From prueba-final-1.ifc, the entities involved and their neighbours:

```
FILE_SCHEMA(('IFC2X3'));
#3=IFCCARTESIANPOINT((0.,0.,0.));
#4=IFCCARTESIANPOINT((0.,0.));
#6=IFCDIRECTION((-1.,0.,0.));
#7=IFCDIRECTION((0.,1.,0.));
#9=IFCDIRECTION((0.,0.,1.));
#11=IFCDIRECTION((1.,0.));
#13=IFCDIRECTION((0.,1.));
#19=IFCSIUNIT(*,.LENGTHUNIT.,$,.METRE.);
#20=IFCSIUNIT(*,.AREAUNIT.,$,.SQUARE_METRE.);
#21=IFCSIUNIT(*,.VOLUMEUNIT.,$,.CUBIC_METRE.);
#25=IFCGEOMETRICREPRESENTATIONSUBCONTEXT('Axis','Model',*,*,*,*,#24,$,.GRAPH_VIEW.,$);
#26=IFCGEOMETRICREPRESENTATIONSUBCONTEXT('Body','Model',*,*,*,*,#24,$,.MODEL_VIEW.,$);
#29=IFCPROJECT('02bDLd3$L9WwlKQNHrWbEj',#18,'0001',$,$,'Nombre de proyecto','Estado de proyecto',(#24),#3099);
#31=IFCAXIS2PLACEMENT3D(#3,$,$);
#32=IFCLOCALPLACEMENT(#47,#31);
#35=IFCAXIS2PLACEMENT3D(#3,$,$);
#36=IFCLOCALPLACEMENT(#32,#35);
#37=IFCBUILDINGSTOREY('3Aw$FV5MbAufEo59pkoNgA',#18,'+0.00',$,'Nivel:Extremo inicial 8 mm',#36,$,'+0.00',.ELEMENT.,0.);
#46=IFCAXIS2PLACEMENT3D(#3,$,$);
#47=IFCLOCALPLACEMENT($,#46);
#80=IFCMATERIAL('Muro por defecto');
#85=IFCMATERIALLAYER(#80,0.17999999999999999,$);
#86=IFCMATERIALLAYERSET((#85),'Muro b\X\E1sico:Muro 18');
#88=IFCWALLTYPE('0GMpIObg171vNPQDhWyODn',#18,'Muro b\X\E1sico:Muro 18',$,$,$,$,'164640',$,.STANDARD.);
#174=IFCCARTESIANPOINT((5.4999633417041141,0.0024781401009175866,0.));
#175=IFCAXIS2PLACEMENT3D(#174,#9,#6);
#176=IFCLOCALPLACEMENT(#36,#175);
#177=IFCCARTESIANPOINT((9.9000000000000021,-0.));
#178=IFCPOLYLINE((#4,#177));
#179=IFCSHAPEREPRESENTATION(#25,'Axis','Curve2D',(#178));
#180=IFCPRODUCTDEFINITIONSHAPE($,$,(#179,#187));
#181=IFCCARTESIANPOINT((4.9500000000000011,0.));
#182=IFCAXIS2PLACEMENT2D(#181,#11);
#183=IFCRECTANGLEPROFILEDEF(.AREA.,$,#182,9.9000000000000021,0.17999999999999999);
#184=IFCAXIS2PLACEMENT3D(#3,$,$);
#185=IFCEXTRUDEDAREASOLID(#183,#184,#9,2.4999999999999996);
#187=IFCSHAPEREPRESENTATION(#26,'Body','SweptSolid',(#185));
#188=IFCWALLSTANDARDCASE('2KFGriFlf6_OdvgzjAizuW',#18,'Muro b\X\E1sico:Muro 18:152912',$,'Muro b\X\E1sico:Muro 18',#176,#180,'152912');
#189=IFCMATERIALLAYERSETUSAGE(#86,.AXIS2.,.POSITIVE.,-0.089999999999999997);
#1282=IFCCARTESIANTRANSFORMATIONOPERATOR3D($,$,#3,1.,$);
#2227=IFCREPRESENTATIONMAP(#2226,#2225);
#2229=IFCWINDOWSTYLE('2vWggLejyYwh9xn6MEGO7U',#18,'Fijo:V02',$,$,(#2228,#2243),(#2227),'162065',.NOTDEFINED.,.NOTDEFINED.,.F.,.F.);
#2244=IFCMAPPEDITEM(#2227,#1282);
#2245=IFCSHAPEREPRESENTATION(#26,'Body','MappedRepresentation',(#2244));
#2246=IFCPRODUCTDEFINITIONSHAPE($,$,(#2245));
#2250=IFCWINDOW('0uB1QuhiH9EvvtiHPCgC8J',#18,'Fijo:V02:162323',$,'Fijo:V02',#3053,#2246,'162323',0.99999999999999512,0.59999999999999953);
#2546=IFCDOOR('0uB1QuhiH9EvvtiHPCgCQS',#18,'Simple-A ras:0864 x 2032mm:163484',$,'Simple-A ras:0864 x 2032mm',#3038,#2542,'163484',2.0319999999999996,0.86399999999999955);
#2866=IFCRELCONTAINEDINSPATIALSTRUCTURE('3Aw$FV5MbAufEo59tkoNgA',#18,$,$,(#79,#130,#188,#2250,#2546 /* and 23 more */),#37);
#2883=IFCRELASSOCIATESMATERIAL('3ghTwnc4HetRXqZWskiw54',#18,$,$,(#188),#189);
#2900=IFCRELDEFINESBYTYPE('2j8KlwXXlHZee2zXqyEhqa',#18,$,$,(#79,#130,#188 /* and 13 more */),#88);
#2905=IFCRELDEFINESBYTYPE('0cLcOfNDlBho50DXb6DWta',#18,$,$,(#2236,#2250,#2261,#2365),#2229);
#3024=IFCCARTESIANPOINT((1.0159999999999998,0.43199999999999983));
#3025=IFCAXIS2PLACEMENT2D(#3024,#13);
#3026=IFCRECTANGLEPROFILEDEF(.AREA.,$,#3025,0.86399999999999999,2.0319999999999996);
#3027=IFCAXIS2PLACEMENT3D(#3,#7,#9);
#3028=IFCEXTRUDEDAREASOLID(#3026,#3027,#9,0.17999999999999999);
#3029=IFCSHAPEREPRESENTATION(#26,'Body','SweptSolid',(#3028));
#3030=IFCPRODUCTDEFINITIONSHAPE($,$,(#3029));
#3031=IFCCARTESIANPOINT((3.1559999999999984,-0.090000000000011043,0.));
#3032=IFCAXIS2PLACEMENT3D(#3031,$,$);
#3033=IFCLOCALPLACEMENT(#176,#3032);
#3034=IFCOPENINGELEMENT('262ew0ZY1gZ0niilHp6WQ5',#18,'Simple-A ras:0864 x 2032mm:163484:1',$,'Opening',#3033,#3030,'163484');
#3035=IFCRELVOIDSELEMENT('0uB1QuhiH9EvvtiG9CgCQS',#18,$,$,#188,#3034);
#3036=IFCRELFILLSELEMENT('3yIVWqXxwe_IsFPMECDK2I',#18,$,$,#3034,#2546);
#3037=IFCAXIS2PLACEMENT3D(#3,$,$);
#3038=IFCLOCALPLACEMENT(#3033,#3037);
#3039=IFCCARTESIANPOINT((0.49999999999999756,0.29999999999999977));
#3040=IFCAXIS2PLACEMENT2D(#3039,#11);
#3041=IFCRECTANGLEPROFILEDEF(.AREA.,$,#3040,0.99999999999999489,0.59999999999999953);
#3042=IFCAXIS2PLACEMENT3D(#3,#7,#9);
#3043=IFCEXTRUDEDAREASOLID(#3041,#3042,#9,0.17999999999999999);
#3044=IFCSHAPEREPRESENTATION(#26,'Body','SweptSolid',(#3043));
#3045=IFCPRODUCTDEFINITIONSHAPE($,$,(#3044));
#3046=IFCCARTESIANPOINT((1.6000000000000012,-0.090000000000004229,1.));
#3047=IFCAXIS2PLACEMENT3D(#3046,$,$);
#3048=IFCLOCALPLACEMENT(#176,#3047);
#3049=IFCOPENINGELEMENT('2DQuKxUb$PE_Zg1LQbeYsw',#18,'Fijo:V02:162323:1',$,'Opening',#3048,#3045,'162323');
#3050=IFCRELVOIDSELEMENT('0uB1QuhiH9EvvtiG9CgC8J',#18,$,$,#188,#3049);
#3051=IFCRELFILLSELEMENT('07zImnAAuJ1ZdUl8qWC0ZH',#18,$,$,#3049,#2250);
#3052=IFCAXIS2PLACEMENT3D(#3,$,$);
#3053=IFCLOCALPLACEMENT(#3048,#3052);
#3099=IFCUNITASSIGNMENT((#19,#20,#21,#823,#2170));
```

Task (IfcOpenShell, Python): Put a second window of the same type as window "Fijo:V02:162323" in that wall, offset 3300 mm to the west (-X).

```python
import ifcopenshell
import ifcopenshell.api.feature
import ifcopenshell.api.geometry
import ifcopenshell.api.root
import ifcopenshell.geom
import ifcopenshell.util.element
import ifcopenshell.util.placement
import ifcopenshell.util.shape

model = ifcopenshell.open("prueba-final-1.ifc")
settings = ifcopenshell.geom.settings()


def volume(element):
    """Net volume in cubic metres, openings subtracted."""
    shape = ifcopenshell.geom.create_shape(settings, element)
    return ifcopenshell.util.shape.get_volume(shape.geometry)


def reuse_history(source, copy):
    """copy_class also copies each property set's owner history, people and application; keep the originals."""
    for rel in copy.IsDefinedBy:
        if rel.is_a("IfcRelDefinesByProperties") and (history := rel.RelatingPropertyDefinition.OwnerHistory):
            rel.RelatingPropertyDefinition.OwnerHistory = source.OwnerHistory
            ifcopenshell.util.element.remove_deep2(model, history)


window = model.by_id(2250)
opening = window.FillsVoids[0].RelatingOpeningElement
wall = opening.VoidsElements[0].RelatingBuildingElement
before = volume(wall)
shift = ifcopenshell.util.placement.get_local_placement(wall.ObjectPlacement)[:3, 0] * 3.3

# copy_class copies the void relationship, type, container and properties, but no geometry.
new_opening = ifcopenshell.api.root.copy_class(model, product=opening)
new_opening.Representation = ifcopenshell.util.element.copy_deep(
    model, opening.Representation, exclude=["IfcGeometricRepresentationContext", "IfcRepresentationMap"]
)
new_opening.Name = "Fijo:V02"
new_opening.Tag = None
new_window = ifcopenshell.api.root.copy_class(model, product=window)
new_window.Representation = ifcopenshell.util.element.copy_deep(
    model, window.Representation, exclude=["IfcGeometricRepresentationContext", "IfcRepresentationMap"]
)
new_window.Name = "Fijo:V02"
new_window.Tag = None
reuse_history(window, new_window)
fills = ifcopenshell.api.feature.add_filling(model, opening=new_opening, element=new_window)
fills.OwnerHistory = new_window.OwnerHistory  # required in IFC2X3

for old, new in ((opening, new_opening), (window, new_window)):
    matrix = ifcopenshell.util.placement.get_local_placement(old.ObjectPlacement)
    matrix[:3, 3] += shift
    ifcopenshell.api.geometry.edit_object_placement(model, product=new, matrix=matrix, is_si=False)

after = volume(wall)

print(f"wall volume {before:.3f} -> {after:.3f} m3")

model.write("prueba-final-1_edited.ifc")
```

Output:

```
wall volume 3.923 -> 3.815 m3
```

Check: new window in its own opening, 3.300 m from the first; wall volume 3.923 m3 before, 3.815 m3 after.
